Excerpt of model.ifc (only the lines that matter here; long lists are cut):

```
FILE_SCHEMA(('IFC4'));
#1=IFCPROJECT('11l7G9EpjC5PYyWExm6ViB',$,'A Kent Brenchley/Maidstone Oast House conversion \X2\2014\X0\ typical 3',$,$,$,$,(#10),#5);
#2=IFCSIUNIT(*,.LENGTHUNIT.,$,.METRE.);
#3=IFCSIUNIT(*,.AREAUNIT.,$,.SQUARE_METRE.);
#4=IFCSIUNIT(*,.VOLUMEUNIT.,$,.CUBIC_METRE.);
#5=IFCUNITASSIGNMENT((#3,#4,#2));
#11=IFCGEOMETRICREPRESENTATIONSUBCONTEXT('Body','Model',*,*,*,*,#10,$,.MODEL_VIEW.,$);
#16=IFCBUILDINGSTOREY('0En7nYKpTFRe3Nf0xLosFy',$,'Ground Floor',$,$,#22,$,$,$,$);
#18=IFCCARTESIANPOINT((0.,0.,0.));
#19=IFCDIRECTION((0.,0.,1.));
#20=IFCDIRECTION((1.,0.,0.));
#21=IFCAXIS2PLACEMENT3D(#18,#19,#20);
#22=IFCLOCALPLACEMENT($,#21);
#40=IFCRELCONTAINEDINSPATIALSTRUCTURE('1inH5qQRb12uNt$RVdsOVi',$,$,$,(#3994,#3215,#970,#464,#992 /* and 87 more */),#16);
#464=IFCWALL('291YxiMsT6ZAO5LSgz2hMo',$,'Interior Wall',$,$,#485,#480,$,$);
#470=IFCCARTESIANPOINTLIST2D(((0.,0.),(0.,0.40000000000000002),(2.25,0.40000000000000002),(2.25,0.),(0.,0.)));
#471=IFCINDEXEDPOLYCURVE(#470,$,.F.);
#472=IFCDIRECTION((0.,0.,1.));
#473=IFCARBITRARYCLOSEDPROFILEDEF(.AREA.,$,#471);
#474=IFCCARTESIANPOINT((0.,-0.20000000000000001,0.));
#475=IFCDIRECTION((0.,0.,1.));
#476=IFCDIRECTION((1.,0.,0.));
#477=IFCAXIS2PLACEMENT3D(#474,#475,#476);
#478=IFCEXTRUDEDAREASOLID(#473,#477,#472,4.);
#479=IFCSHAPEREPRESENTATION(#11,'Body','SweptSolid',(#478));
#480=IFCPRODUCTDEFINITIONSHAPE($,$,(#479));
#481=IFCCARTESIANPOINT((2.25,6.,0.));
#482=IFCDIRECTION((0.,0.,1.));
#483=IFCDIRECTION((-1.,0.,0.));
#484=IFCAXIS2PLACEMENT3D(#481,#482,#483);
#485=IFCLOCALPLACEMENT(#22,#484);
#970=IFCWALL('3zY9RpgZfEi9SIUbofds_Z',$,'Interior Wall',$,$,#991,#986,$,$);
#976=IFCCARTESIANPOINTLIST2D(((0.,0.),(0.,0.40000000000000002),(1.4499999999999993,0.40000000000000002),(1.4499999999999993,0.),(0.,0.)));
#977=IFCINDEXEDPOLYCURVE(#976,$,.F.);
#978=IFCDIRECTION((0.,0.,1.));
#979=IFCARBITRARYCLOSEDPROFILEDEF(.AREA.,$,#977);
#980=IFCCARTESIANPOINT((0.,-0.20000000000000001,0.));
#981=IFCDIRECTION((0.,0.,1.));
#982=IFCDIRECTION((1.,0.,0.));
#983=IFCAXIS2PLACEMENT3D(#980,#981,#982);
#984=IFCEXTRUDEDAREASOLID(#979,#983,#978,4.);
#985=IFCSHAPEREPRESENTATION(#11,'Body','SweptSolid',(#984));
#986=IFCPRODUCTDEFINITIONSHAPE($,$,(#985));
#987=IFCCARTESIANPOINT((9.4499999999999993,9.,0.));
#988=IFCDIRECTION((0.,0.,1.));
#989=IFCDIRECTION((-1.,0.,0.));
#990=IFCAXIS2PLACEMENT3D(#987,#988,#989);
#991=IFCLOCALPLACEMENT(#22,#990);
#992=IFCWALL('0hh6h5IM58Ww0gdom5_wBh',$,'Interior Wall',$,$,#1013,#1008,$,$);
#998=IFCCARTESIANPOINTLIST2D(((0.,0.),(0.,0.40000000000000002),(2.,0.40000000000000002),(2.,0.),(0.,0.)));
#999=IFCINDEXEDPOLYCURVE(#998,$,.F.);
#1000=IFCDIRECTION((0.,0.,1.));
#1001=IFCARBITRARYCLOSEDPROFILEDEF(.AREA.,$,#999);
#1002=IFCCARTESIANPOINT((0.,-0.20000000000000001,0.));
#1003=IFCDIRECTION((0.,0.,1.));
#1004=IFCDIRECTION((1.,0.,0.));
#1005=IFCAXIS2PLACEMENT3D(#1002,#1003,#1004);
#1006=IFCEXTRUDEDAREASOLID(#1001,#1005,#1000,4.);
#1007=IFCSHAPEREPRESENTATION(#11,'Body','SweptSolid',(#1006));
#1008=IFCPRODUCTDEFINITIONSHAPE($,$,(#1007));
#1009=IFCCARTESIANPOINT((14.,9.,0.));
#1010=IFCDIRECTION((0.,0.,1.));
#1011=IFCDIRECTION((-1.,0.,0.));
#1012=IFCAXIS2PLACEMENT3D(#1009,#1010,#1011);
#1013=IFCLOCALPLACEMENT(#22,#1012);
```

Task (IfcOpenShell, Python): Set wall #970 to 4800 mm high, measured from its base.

```python
import ifcopenshell
import ifcopenshell.geom
import ifcopenshell.util.representation
import ifcopenshell.util.shape

model = ifcopenshell.open("model.ifc")
settings = ifcopenshell.geom.settings()


def volume(element):
    """Net volume in cubic metres, openings subtracted."""
    shape = ifcopenshell.geom.create_shape(settings, element)
    return ifcopenshell.util.shape.get_volume(shape.geometry)


wall = model.by_guid("3zY9RpgZfEi9SIUbofds_Z")
before = volume(wall)

body = ifcopenshell.util.representation.get_representation(wall, "Model", "Body")
solid = body.Items[0]
old_height = solid.Depth
solid.Depth = 4.8
after = volume(wall)

print(f"height {old_height:g} -> {solid.Depth:g}, volume {before:.3f} -> {after:.3f} m3")

model.write("model_edited.ifc")
```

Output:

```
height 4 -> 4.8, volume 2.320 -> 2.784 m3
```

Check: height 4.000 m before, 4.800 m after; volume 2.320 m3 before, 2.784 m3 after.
